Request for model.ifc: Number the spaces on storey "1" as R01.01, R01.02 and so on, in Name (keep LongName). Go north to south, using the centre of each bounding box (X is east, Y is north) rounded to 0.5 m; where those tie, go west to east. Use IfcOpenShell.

First a look at what the model holds.

```python
import ifcopenshell
import ifcopenshell.util.element
import ifcopenshell.util.placement

model = ifcopenshell.open("model.ifc")
print(model.schema)
storey = next(s for s in model.by_type("IfcBuildingStorey") if s.Name == "1")
spaces = [e for e in ifcopenshell.util.element.get_decomposition(storey) if e.is_a("IfcSpace")]
for e in sorted(spaces, key=lambda e: e.id()):
    origin = ifcopenshell.util.placement.get_local_placement(e.ObjectPlacement)[:3, 3]
    print(e.id(), e.Name, e.LongName, origin.round(2) + 0.0, sep=" | ")
```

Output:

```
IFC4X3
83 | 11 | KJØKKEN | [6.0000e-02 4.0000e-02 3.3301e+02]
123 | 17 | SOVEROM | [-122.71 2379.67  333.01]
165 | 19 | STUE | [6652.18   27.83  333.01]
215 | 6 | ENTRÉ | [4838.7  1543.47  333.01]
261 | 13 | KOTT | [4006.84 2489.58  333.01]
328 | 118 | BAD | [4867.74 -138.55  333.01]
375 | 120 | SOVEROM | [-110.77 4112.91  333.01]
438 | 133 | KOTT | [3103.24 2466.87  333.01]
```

```python
import ifcopenshell
import ifcopenshell.geom
import ifcopenshell.util.element
import ifcopenshell.util.shape

model = ifcopenshell.open("model.ifc")
settings = ifcopenshell.geom.settings()
settings.set("use-world-coords", True)


def centre(element):
    shape = ifcopenshell.geom.create_shape(settings, element)
    return ifcopenshell.util.shape.get_bbox_centroid(shape.geometry)


storey = next(s for s in model.by_type("IfcBuildingStorey") if s.Name == "1")
spaces = [e for e in ifcopenshell.util.element.get_decomposition(storey) if e.is_a("IfcSpace")]

# Insertion points can sit at a corner or the storey origin, so sort by the geometry (in metres).
centres = {e: centre(e) for e in spaces}
spaces.sort(key=lambda e: (-round(centres[e][1] / 0.5), centres[e][0]))

for i, e in enumerate(spaces, start=1):
    number = f"R01.{i:02d}"
    e.Name = number
    print(e.id(), number)

model.write("model_edited.ifc")
```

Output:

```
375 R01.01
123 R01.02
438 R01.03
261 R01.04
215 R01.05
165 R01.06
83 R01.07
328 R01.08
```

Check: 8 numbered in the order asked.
